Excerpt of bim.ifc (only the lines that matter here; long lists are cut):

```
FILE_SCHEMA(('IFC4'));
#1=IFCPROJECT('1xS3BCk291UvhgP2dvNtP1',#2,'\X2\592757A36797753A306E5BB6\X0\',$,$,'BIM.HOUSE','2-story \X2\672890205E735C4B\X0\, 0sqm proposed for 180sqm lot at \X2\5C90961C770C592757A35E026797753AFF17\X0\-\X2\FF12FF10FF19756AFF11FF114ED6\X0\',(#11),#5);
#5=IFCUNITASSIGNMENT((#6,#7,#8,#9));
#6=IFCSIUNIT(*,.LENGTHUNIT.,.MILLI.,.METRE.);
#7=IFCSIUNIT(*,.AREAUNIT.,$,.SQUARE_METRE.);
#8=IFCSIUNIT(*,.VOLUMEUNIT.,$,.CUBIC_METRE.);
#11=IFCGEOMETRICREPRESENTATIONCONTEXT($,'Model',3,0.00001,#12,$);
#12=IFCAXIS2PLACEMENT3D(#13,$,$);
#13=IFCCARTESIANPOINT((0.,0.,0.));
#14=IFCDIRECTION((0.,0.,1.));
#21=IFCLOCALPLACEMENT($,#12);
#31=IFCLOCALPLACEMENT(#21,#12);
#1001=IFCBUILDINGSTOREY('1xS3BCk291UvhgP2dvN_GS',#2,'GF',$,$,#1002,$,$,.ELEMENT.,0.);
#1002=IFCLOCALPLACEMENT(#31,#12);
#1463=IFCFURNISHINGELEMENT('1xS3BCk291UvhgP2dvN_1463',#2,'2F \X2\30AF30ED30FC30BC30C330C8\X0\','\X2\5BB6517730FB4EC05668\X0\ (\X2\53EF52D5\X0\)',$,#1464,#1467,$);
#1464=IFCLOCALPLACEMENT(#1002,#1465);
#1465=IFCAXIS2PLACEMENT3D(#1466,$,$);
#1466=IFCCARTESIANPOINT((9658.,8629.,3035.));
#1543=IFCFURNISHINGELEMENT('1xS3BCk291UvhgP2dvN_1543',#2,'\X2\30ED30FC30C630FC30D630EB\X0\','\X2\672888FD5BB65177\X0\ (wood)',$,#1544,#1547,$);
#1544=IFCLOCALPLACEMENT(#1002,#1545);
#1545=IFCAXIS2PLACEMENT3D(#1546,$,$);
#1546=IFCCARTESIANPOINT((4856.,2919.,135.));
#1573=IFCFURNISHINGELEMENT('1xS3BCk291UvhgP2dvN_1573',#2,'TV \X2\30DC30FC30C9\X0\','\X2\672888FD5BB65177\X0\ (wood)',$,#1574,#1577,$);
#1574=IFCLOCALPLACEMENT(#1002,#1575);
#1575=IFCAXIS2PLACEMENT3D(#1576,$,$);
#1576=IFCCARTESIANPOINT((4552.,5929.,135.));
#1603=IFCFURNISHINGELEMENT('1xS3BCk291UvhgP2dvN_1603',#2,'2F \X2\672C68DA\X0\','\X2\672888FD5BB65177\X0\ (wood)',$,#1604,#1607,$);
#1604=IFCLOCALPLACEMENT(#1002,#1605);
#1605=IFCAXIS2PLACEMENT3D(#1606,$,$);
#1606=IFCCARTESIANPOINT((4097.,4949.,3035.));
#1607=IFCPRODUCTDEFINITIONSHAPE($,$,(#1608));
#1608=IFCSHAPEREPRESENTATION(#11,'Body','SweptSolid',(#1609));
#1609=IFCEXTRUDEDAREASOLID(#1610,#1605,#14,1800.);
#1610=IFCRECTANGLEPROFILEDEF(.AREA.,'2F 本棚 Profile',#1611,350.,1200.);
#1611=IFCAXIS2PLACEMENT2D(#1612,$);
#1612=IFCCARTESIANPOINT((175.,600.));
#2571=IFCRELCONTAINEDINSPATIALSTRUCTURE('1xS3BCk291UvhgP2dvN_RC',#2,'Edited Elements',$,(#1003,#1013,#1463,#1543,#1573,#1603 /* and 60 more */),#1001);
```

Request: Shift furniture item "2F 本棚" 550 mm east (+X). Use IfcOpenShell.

```python
import ifcopenshell
import ifcopenshell.api.geometry
import ifcopenshell.util.placement

model = ifcopenshell.open("bim.ifc")

item = model.by_id(1603)
matrix = ifcopenshell.util.placement.get_local_placement(item.ObjectPlacement)
matrix[0, 3] += 550.0
ifcopenshell.api.geometry.edit_object_placement(model, product=item, matrix=matrix, is_si=False)

print(ifcopenshell.util.placement.get_local_placement(item.ObjectPlacement).round(3) + 0.0)

model.write("bim_v2.ifc")
```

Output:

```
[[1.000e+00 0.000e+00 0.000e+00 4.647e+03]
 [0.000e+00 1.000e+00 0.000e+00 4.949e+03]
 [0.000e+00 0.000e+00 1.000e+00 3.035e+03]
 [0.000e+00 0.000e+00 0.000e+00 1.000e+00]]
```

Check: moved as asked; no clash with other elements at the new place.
